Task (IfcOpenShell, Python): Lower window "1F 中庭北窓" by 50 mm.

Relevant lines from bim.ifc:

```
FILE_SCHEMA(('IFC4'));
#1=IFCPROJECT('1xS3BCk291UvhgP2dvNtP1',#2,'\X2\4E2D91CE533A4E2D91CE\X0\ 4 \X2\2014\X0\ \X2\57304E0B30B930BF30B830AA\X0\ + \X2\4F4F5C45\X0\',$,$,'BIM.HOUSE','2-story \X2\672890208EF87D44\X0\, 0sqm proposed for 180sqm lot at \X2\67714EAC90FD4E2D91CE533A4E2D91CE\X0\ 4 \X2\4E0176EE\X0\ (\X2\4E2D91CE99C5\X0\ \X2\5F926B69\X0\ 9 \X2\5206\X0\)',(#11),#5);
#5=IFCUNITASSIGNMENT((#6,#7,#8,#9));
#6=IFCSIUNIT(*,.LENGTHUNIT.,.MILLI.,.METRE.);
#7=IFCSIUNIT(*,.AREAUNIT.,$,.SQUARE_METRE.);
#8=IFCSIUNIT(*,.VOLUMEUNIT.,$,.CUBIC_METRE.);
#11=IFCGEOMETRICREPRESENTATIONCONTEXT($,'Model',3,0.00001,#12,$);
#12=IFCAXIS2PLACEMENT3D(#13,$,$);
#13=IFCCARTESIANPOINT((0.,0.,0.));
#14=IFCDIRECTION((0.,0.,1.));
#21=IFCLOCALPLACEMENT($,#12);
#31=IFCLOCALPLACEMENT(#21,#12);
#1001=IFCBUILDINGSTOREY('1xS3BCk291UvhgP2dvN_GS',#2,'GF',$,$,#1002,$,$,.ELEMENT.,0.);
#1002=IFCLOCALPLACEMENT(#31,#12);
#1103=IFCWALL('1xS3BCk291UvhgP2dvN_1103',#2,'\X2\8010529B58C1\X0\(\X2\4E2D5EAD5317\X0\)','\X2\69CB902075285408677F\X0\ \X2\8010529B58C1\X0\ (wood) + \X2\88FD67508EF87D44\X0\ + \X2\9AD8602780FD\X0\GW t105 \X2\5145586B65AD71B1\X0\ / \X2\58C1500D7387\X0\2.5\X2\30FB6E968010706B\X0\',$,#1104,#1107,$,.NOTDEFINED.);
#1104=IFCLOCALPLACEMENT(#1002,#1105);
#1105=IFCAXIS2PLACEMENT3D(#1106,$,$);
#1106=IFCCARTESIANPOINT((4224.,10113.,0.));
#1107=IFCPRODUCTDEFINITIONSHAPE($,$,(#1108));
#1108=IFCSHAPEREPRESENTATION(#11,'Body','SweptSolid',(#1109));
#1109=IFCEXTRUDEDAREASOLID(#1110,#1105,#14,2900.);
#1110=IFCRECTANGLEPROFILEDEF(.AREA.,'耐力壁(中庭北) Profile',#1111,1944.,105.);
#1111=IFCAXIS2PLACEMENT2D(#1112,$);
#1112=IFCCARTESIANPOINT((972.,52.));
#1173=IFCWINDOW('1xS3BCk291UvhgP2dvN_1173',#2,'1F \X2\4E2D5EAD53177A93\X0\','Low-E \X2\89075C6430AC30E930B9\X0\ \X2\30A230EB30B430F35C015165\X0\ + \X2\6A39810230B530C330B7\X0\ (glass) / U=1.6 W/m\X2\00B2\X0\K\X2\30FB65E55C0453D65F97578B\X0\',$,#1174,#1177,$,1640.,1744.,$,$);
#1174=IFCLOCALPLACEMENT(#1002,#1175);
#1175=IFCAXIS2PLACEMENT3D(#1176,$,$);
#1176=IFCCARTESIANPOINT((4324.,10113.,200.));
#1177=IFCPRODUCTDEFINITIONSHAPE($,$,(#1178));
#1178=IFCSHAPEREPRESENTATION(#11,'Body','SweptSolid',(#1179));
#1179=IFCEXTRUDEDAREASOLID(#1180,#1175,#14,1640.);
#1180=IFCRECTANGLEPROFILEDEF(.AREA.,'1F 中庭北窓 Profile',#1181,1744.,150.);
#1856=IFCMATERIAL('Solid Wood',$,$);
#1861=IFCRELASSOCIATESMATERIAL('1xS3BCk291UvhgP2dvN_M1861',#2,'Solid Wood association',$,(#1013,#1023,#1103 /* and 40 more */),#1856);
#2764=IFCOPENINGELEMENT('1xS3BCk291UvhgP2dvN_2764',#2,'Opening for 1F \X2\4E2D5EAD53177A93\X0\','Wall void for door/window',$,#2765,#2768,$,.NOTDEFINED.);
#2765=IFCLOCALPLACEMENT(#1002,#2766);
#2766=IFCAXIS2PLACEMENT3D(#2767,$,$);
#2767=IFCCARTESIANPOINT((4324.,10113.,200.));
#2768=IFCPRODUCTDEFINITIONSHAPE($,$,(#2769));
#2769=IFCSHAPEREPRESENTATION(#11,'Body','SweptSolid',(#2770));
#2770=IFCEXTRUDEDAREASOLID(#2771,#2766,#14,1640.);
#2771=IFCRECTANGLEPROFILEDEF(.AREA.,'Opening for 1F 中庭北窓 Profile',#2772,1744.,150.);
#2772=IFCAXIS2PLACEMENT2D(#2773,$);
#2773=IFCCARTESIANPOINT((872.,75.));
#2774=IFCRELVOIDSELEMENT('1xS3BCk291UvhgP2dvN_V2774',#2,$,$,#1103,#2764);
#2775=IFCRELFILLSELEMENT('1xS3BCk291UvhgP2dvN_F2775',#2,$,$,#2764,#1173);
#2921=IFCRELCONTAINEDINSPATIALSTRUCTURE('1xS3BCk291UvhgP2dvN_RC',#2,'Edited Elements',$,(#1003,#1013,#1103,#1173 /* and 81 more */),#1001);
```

```python
import numpy as np
import ifcopenshell
import ifcopenshell.api.geometry
import ifcopenshell.util.placement
import ifcopenshell.util.unit

model = ifcopenshell.open("bim.ifc")
unit_scale = ifcopenshell.util.unit.calculate_unit_scale(model)

window = model.by_guid("1xS3BCk291UvhgP2dvN_1173")
opening = window.FillsVoids[0].RelatingOpeningElement
dz = -0.05 / unit_scale

shift = np.array([0.0, 0.0, dz])
# The window is not placed relative to its opening, so move both.
for product in (opening, window):
    matrix = ifcopenshell.util.placement.get_local_placement(product.ObjectPlacement)
    matrix[:3, 3] += shift
    ifcopenshell.api.geometry.edit_object_placement(model, product=product, matrix=matrix, is_si=False)

print(f"moved by {dz * unit_scale:+.3f} m")

model.write("bim-out.ifc")
```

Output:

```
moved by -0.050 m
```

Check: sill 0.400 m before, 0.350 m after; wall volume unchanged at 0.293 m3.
